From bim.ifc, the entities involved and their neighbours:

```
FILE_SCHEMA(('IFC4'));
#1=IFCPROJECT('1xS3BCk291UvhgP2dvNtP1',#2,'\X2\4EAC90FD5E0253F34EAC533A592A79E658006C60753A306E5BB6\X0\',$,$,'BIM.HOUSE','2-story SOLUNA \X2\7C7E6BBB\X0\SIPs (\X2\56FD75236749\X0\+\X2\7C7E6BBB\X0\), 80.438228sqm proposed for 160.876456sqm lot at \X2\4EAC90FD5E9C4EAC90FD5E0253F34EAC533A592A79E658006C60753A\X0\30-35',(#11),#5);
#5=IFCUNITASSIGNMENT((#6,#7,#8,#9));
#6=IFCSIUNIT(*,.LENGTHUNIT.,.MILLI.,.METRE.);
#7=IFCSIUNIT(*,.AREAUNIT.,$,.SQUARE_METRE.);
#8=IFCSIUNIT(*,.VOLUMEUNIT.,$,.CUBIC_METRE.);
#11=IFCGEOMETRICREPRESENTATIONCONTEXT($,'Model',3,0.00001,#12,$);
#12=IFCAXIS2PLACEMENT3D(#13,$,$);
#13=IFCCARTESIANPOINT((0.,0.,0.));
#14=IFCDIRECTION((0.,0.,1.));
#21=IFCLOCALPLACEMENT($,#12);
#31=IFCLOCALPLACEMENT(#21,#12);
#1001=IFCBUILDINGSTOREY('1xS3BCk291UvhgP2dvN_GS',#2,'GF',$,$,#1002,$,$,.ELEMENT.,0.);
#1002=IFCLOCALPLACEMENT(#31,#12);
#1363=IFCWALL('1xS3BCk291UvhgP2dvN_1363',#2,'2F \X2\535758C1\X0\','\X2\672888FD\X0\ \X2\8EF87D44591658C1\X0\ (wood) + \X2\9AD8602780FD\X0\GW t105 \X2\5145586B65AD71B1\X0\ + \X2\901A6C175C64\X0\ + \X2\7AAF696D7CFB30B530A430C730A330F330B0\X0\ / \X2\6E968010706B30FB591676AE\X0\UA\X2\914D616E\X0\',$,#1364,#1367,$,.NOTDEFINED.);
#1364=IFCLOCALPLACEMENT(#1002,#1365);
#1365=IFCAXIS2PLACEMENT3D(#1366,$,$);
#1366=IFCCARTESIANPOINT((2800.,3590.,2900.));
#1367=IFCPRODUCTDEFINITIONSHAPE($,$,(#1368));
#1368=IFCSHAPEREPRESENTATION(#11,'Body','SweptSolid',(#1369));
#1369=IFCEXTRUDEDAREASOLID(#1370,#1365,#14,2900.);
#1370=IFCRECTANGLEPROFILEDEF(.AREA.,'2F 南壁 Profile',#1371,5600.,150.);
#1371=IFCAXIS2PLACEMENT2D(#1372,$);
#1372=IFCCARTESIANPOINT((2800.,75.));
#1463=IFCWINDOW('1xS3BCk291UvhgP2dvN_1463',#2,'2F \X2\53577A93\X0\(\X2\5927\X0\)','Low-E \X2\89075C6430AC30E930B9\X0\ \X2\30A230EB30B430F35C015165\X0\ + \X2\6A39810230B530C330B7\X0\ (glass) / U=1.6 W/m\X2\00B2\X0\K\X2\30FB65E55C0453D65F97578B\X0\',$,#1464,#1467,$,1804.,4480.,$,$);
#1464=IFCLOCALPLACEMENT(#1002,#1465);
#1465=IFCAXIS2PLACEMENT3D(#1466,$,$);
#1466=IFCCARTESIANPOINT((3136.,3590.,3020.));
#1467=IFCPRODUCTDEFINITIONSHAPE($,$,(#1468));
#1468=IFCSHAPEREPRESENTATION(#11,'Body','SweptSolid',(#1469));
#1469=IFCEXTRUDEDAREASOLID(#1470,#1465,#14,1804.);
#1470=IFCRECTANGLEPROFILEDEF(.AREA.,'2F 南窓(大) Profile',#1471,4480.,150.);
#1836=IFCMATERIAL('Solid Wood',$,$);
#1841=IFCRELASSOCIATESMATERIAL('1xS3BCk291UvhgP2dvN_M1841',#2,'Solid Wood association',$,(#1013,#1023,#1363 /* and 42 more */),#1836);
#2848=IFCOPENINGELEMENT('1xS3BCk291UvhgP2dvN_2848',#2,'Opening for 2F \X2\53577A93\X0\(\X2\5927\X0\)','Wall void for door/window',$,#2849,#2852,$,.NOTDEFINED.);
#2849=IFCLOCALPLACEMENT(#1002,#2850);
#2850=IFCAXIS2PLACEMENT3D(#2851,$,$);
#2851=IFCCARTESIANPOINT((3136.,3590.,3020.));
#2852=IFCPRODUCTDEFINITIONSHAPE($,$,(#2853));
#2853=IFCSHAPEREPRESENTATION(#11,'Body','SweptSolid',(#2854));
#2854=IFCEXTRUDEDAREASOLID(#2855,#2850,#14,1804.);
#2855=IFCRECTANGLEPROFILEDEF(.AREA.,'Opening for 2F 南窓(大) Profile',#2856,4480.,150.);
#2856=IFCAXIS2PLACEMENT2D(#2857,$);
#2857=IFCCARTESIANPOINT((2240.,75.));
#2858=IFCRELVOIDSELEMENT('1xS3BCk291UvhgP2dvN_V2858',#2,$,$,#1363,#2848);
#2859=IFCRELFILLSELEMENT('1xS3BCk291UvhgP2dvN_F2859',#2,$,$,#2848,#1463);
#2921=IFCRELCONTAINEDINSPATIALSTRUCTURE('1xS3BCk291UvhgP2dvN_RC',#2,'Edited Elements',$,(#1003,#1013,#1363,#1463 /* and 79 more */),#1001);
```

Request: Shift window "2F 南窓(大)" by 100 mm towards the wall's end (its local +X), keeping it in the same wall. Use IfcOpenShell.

```python
import ifcopenshell
import ifcopenshell.api.geometry
import ifcopenshell.util.placement

model = ifcopenshell.open("bim.ifc")

window = model.by_id(1463)
opening = window.FillsVoids[0].RelatingOpeningElement
wall = opening.VoidsElements[0].RelatingBuildingElement

wall_matrix = ifcopenshell.util.placement.get_local_placement(wall.ObjectPlacement)
shift = wall_matrix[:3, 0] * 100.0
before = ifcopenshell.util.placement.get_local_placement(window.ObjectPlacement)[:3, 3].copy()

# The window is not placed relative to its opening, so move both.
for product in (opening, window):
    matrix = ifcopenshell.util.placement.get_local_placement(product.ObjectPlacement)
    matrix[:3, 3] += shift
    ifcopenshell.api.geometry.edit_object_placement(model, product=product, matrix=matrix, is_si=False)

after = ifcopenshell.util.placement.get_local_placement(window.ObjectPlacement)[:3, 3]
print("window moved by", (after - before).round(3) + 0.0)

model.write("bim_edited.ifc")
```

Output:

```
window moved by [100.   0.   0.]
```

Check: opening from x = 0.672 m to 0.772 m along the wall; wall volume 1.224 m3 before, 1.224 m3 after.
